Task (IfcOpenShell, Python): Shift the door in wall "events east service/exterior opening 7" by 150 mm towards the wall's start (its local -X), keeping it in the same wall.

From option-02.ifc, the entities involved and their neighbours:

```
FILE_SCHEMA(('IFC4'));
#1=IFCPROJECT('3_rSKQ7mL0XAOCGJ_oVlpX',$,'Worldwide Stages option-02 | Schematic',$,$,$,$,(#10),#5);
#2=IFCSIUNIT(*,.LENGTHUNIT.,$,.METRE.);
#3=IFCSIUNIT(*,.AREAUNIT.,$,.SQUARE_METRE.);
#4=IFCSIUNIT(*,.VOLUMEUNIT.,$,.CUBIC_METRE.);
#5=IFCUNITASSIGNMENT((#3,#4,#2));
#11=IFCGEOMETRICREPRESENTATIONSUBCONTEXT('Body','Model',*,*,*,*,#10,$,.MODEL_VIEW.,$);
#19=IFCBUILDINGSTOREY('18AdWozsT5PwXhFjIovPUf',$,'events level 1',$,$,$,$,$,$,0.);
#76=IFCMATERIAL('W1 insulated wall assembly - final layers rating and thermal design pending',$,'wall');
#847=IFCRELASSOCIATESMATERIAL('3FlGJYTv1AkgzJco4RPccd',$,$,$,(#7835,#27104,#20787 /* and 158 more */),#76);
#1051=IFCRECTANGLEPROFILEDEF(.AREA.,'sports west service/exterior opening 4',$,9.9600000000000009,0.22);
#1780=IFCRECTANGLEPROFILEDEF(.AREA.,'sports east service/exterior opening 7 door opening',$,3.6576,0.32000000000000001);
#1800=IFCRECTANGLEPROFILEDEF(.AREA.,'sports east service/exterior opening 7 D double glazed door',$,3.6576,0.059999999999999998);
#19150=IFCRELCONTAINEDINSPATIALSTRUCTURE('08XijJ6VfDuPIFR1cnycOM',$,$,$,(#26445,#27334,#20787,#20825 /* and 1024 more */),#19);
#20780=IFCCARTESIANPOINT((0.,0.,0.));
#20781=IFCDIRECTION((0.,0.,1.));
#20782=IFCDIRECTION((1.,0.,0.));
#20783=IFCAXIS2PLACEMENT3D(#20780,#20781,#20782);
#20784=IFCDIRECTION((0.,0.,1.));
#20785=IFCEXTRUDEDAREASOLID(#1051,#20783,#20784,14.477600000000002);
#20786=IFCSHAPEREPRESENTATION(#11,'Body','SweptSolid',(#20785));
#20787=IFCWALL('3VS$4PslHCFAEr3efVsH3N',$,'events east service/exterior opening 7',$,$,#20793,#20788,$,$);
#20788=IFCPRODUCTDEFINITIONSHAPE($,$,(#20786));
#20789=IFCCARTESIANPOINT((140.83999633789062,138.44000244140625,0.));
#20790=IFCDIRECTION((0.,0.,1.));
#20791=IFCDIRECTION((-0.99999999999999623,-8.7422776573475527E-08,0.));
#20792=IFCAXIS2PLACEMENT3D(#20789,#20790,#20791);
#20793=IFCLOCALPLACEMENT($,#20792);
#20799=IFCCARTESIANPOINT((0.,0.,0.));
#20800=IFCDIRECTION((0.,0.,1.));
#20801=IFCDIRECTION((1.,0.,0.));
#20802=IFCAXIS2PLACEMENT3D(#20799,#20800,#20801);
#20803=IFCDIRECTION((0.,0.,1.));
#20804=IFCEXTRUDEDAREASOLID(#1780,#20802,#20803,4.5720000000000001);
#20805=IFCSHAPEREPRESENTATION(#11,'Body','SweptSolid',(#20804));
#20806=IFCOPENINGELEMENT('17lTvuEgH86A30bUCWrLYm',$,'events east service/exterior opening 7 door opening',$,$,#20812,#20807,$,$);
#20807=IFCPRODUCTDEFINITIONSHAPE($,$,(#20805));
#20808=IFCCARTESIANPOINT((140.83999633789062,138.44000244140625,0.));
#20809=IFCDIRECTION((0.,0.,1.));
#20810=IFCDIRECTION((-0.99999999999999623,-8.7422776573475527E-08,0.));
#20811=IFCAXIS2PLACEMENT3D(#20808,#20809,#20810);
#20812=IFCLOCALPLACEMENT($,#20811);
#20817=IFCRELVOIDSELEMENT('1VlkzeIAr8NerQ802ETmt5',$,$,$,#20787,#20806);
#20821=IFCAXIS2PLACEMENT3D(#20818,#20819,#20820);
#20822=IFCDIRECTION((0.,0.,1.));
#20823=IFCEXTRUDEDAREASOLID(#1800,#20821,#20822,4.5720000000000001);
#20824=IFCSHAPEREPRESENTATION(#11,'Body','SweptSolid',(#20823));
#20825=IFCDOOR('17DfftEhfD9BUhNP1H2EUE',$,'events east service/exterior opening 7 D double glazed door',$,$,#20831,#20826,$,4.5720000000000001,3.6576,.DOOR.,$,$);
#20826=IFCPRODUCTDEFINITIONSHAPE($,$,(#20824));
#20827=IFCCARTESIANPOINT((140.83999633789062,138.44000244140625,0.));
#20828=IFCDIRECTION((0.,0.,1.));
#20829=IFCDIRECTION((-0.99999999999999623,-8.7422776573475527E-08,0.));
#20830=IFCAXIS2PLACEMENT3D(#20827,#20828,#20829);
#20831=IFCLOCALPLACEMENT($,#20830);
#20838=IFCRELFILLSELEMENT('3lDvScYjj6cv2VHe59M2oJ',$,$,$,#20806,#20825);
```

```python
import ifcopenshell
import ifcopenshell.api.geometry
import ifcopenshell.util.placement
import ifcopenshell.util.unit

model = ifcopenshell.open("option-02.ifc")
unit_scale = ifcopenshell.util.unit.calculate_unit_scale(model)

door = model.by_guid("17DfftEhfD9BUhNP1H2EUE")
opening = door.FillsVoids[0].RelatingOpeningElement
wall = opening.VoidsElements[0].RelatingBuildingElement

wall_matrix = ifcopenshell.util.placement.get_local_placement(wall.ObjectPlacement)
shift = wall_matrix[:3, 0] * -0.15 / unit_scale
before = ifcopenshell.util.placement.get_local_placement(door.ObjectPlacement)[:3, 3].copy()

# The door is not placed relative to its opening, so move both.
for product in (opening, door):
    matrix = ifcopenshell.util.placement.get_local_placement(product.ObjectPlacement)
    matrix[:3, 3] += shift
    ifcopenshell.api.geometry.edit_object_placement(model, product=product, matrix=matrix, is_si=False)

after = ifcopenshell.util.placement.get_local_placement(door.ObjectPlacement)[:3, 3]
print("door moved by", (after - before).round(3) + 0.0)

model.write("option-02_rev.ifc")
```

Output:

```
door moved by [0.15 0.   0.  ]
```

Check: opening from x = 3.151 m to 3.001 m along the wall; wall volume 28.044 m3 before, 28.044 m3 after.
